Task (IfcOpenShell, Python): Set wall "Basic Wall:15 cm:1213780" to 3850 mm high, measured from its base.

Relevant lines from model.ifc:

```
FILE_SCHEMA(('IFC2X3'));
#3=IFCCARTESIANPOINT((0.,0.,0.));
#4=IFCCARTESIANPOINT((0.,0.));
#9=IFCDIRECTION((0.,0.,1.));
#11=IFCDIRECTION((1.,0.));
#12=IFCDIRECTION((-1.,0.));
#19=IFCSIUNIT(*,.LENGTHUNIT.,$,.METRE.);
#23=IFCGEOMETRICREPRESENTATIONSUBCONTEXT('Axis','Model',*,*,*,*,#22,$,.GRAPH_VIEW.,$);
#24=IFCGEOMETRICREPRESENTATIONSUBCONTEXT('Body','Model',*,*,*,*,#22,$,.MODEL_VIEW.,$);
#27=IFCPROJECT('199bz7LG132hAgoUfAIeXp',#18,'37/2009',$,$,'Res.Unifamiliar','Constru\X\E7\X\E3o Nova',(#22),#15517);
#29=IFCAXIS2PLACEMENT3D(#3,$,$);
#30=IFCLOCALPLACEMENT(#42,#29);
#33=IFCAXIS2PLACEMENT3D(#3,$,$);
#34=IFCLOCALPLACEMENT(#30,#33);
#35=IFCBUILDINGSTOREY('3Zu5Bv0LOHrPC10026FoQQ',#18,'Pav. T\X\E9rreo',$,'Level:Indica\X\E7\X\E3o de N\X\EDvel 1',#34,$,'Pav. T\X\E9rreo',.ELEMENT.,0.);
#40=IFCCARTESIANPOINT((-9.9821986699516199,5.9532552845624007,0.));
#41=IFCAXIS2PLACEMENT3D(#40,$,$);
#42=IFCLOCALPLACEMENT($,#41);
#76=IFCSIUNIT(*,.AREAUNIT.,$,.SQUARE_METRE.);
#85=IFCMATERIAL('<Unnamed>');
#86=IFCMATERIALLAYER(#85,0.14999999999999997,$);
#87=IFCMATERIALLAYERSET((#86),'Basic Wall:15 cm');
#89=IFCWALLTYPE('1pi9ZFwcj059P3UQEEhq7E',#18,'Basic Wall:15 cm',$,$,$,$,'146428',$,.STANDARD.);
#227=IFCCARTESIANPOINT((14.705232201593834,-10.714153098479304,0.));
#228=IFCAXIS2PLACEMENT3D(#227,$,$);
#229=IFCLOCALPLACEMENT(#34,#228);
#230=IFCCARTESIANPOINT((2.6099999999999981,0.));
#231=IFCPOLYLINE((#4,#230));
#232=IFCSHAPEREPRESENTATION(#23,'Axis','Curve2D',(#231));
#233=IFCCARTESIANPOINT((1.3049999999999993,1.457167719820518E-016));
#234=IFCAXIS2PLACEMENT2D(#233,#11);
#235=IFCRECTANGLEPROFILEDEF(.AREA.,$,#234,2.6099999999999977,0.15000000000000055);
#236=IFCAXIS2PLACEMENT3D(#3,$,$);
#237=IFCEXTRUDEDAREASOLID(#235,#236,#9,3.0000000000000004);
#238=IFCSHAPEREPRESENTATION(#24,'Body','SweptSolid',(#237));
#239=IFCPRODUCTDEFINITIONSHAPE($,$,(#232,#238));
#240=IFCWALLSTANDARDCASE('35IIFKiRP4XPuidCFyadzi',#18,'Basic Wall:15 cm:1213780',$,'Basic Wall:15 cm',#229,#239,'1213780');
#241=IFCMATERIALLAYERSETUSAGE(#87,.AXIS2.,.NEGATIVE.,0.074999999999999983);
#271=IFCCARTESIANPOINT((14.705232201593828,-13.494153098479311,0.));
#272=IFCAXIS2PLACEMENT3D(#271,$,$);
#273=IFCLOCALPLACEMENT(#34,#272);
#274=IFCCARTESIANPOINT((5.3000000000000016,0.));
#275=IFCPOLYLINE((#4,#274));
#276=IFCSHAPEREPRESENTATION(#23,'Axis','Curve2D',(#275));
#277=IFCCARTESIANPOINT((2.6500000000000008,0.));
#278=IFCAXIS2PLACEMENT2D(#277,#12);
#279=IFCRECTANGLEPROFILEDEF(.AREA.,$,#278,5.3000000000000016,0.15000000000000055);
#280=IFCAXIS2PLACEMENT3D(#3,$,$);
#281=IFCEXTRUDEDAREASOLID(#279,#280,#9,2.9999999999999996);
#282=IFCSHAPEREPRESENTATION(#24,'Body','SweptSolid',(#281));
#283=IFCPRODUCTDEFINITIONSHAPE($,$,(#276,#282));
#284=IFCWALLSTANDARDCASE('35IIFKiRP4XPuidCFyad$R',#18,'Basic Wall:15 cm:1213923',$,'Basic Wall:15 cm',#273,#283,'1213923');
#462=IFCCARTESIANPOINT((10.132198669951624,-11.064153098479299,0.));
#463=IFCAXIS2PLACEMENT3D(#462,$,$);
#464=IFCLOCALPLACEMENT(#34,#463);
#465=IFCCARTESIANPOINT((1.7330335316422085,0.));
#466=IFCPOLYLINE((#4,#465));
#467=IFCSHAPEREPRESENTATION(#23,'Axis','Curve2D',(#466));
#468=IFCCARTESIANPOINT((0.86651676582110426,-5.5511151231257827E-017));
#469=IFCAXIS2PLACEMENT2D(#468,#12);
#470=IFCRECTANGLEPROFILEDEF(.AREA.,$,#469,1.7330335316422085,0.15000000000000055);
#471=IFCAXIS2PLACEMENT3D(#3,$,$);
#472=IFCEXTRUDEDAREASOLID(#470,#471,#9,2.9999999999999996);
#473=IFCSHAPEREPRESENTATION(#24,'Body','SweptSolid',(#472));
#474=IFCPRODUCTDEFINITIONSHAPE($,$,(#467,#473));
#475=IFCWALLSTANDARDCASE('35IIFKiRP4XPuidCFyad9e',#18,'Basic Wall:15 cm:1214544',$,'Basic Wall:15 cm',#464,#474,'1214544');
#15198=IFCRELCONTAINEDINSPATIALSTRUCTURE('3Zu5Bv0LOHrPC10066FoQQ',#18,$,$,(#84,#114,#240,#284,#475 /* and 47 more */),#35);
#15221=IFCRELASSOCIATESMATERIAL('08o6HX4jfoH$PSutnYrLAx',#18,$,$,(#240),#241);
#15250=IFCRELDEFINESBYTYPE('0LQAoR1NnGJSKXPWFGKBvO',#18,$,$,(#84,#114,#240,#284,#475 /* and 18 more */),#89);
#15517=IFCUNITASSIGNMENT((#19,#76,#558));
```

```python
import ifcopenshell
import ifcopenshell.geom
import ifcopenshell.util.representation
import ifcopenshell.util.shape

model = ifcopenshell.open("model.ifc")
settings = ifcopenshell.geom.settings()


def volume(element):
    """Net volume in cubic metres, openings subtracted."""
    shape = ifcopenshell.geom.create_shape(settings, element)
    return ifcopenshell.util.shape.get_volume(shape.geometry)


wall = model.by_guid("35IIFKiRP4XPuidCFyadzi")
before = volume(wall)

body = ifcopenshell.util.representation.get_representation(wall, "Model", "Body")
solid = body.Items[0]
old_height = solid.Depth
solid.Depth = 3.85
after = volume(wall)

print(f"height {old_height:g} -> {solid.Depth:g}, volume {before:.3f} -> {after:.3f} m3")

model.write("model_rev.ifc")
```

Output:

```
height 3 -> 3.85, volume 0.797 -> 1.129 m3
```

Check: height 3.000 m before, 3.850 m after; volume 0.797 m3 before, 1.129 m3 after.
